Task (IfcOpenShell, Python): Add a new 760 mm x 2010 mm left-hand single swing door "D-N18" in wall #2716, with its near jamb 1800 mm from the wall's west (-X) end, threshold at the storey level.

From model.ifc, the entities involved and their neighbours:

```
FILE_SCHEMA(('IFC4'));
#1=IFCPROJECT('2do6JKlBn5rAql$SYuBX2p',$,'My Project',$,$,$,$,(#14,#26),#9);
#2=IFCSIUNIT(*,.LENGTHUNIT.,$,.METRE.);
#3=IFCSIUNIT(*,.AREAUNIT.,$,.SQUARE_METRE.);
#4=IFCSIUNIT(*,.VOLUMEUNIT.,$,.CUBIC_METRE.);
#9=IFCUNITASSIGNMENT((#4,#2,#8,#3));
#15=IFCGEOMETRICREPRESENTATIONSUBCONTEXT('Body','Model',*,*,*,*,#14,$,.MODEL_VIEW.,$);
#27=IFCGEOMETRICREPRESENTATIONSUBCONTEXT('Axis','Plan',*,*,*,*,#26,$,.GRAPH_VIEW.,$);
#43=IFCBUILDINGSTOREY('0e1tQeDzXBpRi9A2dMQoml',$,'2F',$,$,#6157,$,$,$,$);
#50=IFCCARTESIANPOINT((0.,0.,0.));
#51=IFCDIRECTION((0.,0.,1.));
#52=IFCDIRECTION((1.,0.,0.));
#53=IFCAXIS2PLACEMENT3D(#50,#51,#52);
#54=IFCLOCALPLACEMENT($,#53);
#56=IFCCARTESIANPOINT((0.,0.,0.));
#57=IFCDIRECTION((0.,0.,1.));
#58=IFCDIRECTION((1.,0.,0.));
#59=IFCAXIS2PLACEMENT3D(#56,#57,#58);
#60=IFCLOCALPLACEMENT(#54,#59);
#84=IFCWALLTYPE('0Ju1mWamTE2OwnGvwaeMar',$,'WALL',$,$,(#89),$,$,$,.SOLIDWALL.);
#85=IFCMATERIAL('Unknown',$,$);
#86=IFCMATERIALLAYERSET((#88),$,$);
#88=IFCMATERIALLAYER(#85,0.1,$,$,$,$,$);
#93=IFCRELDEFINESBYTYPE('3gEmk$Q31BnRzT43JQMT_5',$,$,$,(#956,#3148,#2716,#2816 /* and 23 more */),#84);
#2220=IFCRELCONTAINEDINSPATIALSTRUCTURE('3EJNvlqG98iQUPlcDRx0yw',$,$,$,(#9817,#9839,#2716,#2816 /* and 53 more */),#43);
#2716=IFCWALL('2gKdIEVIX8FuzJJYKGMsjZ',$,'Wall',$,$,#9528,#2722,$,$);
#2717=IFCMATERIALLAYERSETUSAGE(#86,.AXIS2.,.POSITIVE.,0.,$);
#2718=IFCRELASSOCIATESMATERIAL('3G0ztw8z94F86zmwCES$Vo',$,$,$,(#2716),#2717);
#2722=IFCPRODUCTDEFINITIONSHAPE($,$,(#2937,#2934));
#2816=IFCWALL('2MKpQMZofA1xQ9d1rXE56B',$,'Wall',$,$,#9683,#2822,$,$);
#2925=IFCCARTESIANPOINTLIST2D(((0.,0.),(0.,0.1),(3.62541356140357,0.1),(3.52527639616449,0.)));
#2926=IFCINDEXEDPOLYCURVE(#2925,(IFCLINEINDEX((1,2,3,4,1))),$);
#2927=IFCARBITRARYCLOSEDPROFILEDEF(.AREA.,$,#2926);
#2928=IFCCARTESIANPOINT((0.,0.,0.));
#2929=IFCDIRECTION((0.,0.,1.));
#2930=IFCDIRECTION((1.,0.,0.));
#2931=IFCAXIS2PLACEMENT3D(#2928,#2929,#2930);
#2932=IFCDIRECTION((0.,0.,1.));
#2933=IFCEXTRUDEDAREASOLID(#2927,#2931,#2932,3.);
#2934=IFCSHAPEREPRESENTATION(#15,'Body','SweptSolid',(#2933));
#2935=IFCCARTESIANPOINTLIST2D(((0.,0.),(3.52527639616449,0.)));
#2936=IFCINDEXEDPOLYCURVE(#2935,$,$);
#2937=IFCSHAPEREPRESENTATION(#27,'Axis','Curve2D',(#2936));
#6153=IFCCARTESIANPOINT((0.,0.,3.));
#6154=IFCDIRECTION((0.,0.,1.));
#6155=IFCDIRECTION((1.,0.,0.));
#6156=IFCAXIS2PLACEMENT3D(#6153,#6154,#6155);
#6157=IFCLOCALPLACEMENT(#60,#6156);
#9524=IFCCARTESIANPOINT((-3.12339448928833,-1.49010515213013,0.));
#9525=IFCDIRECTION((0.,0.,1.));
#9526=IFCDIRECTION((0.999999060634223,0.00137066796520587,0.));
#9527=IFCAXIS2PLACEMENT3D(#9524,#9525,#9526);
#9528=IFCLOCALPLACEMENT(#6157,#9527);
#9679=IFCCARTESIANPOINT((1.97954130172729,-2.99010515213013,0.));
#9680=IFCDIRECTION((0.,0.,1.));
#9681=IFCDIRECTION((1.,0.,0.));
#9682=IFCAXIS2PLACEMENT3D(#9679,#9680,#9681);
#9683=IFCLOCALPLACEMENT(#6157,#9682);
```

```python
import numpy as np
import ifcopenshell
import ifcopenshell.api.feature
import ifcopenshell.api.geometry
import ifcopenshell.api.root
import ifcopenshell.api.spatial
import ifcopenshell.geom
import ifcopenshell.util.element
import ifcopenshell.util.placement
import ifcopenshell.util.representation
import ifcopenshell.util.shape
import ifcopenshell.util.unit

model = ifcopenshell.open("model.ifc")
unit_scale = ifcopenshell.util.unit.calculate_unit_scale(model)
settings = ifcopenshell.geom.settings()


def volume(element):
    """Net volume in cubic metres, openings subtracted."""
    shape = ifcopenshell.geom.create_shape(settings, element)
    return ifcopenshell.util.shape.get_volume(shape.geometry)


wall = model.by_guid("2gKdIEVIX8FuzJJYKGMsjZ")
storey = ifcopenshell.util.element.get_container(wall, ifc_class="IfcBuildingStorey")
context = ifcopenshell.util.representation.get_context(model, "Model", "Body", "MODEL_VIEW")
before = volume(wall)

width, height, from_end, sill = 0.76, 2.01, 1.8, 0.0  # metres

# The wall runs along its own X axis, and the end named is its -X end.
wall_shape = ifcopenshell.geom.create_shape(settings, wall)
x, y, z = ifcopenshell.util.shape.get_vertices(wall_shape.geometry).T
start = x.min() + from_end
face, thickness = float(y.min()), float(y.max() - y.min())
wall_matrix = ifcopenshell.util.placement.get_local_placement(wall.ObjectPlacement)
level = ifcopenshell.util.placement.get_local_placement(storey.ObjectPlacement)[2, 3]


def in_wall(x, y):
    """Placement at x, y metres in the wall's axes, at sill height."""
    matrix = wall_matrix.copy()
    matrix[:, 3] = wall_matrix @ np.array([x / unit_scale, y / unit_scale, 0.0, 1.0])
    matrix[2, 3] = level + sill / unit_scale
    return matrix


# Opening: a box that overshoots both wall faces by 50 mm.
opening = ifcopenshell.api.root.create_entity(model, ifc_class="IfcOpeningElement", predefined_type="OPENING")
box = ifcopenshell.api.geometry.add_wall_representation(
    model, context=context, length=width, height=height, thickness=thickness + 0.1
)
ifcopenshell.api.geometry.assign_representation(model, product=opening, representation=box)
ifcopenshell.api.geometry.edit_object_placement(model, product=opening, matrix=in_wall(start, face - 0.05), is_si=False)
ifcopenshell.api.feature.add_feature(model, feature=opening, element=wall)

door = ifcopenshell.api.root.create_entity(model, ifc_class="IfcDoor", name="D-N18", predefined_type="DOOR")
door.OverallWidth, door.OverallHeight = width / unit_scale, height / unit_scale
door.OperationType = "SINGLE_SWING_LEFT"
body = ifcopenshell.api.geometry.add_door_representation(
    model,
    context=context,
    overall_width=door.OverallWidth,
    overall_height=door.OverallHeight,
    operation_type="SINGLE_SWING_LEFT",
    lining_properties={"LiningDepth": thickness / unit_scale, "ThresholdDepth": thickness / unit_scale},
)
ifcopenshell.api.geometry.assign_representation(model, product=door, representation=body)
ifcopenshell.api.spatial.assign_container(model, products=[door], relating_structure=storey)
ifcopenshell.api.feature.add_filling(model, opening=opening, element=door)

# The lining spans the wall, so the door starts at the wall face.
ifcopenshell.api.geometry.edit_object_placement(model, product=door, matrix=in_wall(start, face), is_si=False)

after = volume(wall)

print(f"wall volume {before:.3f} -> {after:.3f} m3")

model.write("model-out.ifc")
```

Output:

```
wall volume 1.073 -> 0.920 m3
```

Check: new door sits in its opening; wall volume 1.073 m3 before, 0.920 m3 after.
